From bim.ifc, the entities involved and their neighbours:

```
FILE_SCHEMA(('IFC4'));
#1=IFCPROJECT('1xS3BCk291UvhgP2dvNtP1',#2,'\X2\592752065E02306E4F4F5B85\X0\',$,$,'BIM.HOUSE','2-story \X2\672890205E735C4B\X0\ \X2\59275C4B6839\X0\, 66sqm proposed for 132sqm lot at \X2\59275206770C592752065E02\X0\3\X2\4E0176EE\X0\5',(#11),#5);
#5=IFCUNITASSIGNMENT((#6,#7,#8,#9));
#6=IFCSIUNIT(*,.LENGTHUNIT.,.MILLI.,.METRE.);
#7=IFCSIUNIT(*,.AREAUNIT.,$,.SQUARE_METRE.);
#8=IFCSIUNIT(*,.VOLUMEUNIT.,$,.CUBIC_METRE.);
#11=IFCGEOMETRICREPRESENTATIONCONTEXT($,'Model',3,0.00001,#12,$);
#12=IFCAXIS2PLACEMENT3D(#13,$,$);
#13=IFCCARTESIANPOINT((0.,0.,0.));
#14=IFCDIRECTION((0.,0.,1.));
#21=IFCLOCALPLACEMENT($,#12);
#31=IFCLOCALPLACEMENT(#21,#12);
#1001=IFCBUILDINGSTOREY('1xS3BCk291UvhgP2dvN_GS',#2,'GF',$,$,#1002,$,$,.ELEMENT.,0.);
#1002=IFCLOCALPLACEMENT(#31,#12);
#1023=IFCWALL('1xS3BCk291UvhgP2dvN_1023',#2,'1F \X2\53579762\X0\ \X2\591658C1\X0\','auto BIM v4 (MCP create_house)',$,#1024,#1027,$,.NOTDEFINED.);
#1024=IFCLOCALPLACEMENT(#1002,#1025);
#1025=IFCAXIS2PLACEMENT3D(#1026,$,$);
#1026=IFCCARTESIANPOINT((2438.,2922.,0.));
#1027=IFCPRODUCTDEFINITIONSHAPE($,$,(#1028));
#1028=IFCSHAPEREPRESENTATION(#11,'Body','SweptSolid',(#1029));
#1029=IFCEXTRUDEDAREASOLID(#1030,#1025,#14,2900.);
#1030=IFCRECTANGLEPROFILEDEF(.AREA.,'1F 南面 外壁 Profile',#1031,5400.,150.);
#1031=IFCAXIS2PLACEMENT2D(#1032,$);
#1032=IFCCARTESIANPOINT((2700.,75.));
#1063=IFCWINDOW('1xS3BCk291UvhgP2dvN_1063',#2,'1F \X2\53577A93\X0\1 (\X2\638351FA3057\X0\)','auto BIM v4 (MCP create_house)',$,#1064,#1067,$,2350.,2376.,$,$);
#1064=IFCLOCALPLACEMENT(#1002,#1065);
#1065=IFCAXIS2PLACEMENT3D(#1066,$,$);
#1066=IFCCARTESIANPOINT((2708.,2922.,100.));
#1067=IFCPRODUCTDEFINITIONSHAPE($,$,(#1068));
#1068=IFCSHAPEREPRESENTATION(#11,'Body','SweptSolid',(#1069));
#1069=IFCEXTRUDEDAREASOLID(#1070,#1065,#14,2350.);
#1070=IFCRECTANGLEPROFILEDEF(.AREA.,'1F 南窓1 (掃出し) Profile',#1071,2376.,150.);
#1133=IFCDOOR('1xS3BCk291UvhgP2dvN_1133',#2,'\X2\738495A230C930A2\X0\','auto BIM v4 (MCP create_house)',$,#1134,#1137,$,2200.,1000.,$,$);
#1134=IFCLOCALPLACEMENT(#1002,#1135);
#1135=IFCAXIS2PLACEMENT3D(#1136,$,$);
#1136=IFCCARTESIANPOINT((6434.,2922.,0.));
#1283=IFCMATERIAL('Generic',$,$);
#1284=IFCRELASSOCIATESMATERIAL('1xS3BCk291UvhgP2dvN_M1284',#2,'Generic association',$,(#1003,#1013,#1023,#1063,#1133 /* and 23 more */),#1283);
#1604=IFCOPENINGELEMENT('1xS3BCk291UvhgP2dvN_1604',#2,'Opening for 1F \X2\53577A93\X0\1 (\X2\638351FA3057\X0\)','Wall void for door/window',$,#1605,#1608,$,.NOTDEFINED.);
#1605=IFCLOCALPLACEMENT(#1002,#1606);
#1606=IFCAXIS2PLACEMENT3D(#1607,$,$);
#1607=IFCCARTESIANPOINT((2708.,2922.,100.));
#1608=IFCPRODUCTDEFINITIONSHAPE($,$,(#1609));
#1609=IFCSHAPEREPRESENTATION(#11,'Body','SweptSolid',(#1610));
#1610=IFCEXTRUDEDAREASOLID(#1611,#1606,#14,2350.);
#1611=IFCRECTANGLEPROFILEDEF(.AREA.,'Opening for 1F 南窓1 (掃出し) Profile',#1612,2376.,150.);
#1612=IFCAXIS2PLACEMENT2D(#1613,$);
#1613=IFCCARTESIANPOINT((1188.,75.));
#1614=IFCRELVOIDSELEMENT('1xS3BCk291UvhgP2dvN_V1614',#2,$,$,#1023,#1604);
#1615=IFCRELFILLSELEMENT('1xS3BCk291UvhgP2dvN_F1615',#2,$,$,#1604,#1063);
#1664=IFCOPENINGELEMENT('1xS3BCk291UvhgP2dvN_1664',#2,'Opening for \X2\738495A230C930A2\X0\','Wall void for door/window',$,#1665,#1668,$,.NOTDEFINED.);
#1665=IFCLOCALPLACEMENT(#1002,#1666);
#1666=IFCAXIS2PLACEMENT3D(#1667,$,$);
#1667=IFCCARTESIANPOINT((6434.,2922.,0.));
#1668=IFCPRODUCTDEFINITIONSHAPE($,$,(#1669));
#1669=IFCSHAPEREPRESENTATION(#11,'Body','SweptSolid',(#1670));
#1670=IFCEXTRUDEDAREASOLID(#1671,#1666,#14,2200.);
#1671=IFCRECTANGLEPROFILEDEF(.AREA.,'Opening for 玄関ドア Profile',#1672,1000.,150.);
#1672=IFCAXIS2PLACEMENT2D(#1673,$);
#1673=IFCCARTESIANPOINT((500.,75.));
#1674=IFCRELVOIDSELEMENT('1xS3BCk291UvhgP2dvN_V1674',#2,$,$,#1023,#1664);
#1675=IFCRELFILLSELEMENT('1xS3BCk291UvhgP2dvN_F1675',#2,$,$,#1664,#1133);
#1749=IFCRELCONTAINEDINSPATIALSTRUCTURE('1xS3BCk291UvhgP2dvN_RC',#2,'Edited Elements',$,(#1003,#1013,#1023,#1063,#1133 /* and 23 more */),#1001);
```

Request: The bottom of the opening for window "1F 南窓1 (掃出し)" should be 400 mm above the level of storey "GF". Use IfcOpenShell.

```python
import numpy as np
import ifcopenshell
import ifcopenshell.api.geometry
import ifcopenshell.geom
import ifcopenshell.util.element
import ifcopenshell.util.placement
import ifcopenshell.util.shape
import ifcopenshell.util.unit

model = ifcopenshell.open("bim.ifc")
unit_scale = ifcopenshell.util.unit.calculate_unit_scale(model)

window = model.by_id(1063)
opening = window.FillsVoids[0].RelatingOpeningElement
storey = ifcopenshell.util.element.get_container(window, ifc_class="IfcBuildingStorey")
level = ifcopenshell.util.placement.get_local_placement(storey.ObjectPlacement)[2, 3]

# The opening's origin need not be at the sill, so measure its lowest point.
shape = ifcopenshell.geom.create_shape(ifcopenshell.geom.settings(), opening)
bottom = ifcopenshell.util.shape.get_shape_bottom_elevation(shape, shape.geometry) / unit_scale
dz = level + 0.4 / unit_scale - bottom

shift = np.array([0.0, 0.0, dz])
# The window is not placed relative to its opening, so move both.
for product in (opening, window):
    matrix = ifcopenshell.util.placement.get_local_placement(product.ObjectPlacement)
    matrix[:3, 3] += shift
    ifcopenshell.api.geometry.edit_object_placement(model, product=product, matrix=matrix, is_si=False)

print(f"moved by {dz * unit_scale:+.3f} m")

model.write("bim_rev.ifc")
```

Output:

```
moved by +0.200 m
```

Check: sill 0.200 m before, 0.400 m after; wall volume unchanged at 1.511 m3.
